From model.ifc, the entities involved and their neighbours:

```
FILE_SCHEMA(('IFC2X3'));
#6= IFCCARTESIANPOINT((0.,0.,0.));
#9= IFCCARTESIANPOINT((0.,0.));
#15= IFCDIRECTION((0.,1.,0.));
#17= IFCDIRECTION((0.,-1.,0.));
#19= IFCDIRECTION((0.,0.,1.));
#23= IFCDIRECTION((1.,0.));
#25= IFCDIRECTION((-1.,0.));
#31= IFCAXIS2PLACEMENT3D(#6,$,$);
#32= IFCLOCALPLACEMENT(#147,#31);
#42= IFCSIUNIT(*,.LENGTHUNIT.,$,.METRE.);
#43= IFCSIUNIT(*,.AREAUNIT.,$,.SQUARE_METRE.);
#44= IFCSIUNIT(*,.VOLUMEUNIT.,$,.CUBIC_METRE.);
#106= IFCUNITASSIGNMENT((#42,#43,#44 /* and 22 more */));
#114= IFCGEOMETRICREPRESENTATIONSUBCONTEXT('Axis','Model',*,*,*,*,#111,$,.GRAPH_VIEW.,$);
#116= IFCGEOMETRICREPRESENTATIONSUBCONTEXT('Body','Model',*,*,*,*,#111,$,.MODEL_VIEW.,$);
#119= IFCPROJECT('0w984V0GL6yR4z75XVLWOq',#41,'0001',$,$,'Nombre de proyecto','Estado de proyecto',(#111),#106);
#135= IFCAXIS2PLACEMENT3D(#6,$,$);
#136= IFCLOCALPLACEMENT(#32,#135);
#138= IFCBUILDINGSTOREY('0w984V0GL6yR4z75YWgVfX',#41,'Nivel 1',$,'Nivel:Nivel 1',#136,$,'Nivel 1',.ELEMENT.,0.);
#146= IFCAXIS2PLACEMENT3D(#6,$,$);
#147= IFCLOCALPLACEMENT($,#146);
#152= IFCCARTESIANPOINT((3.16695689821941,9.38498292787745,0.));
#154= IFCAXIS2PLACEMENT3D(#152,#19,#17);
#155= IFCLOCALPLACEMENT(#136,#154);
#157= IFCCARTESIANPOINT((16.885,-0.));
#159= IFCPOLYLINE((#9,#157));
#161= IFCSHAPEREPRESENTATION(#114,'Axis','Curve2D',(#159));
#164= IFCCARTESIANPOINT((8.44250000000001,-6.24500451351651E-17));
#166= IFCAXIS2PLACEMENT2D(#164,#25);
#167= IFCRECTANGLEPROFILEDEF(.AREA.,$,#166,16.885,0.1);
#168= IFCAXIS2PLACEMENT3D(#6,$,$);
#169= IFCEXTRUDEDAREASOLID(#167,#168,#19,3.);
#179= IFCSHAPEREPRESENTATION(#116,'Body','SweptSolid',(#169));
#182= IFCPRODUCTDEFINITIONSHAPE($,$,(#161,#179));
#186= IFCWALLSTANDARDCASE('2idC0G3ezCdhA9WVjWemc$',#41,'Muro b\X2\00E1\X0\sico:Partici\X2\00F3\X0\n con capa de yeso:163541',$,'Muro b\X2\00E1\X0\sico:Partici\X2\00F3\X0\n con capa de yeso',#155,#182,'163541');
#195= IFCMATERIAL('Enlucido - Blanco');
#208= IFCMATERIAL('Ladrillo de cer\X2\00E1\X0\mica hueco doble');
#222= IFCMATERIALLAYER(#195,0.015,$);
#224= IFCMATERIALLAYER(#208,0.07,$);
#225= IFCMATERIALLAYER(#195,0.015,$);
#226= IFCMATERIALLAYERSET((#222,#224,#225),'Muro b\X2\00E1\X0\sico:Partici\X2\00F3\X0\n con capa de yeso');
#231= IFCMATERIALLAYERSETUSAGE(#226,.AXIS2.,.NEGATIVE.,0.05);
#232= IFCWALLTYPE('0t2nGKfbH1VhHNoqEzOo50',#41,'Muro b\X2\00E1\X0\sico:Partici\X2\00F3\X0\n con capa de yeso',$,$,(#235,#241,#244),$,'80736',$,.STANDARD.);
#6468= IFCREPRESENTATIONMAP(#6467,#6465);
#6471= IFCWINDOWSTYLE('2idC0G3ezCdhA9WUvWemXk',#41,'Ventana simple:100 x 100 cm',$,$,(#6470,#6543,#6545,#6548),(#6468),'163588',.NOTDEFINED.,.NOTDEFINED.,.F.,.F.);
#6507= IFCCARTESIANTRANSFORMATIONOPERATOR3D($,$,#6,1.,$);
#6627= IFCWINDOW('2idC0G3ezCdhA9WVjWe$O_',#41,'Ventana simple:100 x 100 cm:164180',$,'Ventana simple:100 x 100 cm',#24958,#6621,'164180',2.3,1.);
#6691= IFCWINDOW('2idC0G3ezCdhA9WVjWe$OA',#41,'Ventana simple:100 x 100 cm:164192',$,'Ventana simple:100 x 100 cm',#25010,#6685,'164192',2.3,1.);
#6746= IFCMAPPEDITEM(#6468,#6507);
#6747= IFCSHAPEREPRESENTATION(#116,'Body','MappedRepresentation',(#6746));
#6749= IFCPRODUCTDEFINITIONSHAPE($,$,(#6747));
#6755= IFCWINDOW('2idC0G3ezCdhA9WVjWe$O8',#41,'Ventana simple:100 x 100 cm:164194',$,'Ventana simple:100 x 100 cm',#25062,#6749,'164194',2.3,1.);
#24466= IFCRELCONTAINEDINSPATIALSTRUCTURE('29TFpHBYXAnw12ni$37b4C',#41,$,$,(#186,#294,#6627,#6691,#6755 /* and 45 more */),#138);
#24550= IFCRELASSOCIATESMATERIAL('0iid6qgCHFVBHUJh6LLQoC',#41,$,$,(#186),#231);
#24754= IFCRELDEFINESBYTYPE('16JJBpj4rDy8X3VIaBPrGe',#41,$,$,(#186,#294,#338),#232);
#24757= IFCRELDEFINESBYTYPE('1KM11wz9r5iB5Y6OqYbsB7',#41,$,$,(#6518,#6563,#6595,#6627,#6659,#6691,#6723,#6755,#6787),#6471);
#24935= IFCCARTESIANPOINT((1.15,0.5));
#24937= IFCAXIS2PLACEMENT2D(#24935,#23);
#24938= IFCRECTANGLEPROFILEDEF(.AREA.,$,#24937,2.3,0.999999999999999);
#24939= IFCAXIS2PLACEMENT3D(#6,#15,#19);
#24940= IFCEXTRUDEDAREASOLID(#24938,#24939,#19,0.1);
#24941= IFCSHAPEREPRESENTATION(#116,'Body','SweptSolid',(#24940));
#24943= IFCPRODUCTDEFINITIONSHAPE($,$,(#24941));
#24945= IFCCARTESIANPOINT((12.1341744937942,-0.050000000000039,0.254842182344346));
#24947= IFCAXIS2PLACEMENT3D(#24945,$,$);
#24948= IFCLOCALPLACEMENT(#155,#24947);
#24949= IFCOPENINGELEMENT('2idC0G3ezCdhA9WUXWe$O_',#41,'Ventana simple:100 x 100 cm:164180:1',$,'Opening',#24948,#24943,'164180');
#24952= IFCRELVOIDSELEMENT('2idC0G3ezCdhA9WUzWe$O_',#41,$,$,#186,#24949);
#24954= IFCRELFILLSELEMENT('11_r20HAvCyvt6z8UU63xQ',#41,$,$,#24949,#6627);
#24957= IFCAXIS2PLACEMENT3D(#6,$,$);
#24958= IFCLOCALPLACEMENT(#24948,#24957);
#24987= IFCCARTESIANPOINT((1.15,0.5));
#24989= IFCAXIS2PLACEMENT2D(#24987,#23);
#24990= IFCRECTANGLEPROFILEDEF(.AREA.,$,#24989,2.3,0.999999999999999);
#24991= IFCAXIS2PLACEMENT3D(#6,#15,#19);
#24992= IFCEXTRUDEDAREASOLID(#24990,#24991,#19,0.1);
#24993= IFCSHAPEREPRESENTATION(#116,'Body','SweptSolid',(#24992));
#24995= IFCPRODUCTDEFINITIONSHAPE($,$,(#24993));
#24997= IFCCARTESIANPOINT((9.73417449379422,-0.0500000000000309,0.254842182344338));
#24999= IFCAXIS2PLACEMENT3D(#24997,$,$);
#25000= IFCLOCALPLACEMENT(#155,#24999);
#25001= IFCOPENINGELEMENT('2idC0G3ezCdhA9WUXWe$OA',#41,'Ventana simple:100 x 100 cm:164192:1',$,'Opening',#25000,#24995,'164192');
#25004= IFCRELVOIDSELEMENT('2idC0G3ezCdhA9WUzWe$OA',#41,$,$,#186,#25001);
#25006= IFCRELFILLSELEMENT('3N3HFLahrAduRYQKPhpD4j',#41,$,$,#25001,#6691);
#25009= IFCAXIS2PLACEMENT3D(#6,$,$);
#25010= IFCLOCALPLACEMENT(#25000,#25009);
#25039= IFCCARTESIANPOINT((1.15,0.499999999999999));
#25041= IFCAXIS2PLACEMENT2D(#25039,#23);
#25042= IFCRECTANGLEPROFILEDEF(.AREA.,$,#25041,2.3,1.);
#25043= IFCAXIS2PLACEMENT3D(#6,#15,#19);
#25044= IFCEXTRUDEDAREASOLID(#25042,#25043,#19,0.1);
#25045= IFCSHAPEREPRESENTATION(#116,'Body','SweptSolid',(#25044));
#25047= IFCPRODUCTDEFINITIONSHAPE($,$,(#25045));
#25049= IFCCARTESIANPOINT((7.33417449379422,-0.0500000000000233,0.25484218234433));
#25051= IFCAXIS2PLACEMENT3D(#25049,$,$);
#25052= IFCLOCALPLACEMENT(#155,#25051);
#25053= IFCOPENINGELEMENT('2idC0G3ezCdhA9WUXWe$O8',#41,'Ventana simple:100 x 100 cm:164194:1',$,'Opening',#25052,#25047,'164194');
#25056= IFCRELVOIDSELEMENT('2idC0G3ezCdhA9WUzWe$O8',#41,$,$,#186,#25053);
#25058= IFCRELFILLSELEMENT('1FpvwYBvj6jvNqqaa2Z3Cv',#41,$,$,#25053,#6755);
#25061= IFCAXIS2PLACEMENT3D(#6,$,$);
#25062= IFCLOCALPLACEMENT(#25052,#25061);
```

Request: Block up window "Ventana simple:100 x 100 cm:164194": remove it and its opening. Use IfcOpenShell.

```python
import ifcopenshell
import ifcopenshell.api.feature
import ifcopenshell.api.root
import ifcopenshell.geom
import ifcopenshell.util.shape

model = ifcopenshell.open("model.ifc")
settings = ifcopenshell.geom.settings()


def volume(element):
    """Net volume in cubic metres, openings subtracted."""
    shape = ifcopenshell.geom.create_shape(settings, element)
    return ifcopenshell.util.shape.get_volume(shape.geometry)


window = model.by_guid("2idC0G3ezCdhA9WVjWe$O8")
opening = window.FillsVoids[0].RelatingOpeningElement
wall = opening.VoidsElements[0].RelatingBuildingElement
before = volume(wall)

ifcopenshell.api.root.remove_product(model, product=window)
ifcopenshell.api.feature.remove_feature(model, feature=opening)

after = volume(wall)

print(f"wall volume {before:.3f} -> {after:.3f} m3")

model.write("model_v2.ifc")
```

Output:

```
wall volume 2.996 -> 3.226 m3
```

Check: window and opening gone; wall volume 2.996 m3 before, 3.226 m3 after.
